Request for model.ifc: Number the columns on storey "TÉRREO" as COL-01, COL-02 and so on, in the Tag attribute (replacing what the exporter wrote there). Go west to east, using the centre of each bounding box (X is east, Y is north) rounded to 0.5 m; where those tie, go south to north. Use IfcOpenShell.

First a look at what the model holds.

```python
import ifcopenshell
import ifcopenshell.util.element
import ifcopenshell.util.placement

model = ifcopenshell.open("model.ifc")
print(model.schema)
storey = next(s for s in model.by_type("IfcBuildingStorey") if s.Name == "TÉRREO")
columns = [e for e in ifcopenshell.util.element.get_decomposition(storey) if e.is_a("IfcColumn")]
for e in sorted(columns, key=lambda e: e.id()):
    origin = ifcopenshell.util.placement.get_local_placement(e.ObjectPlacement)[:3, 3]
    print(e.id(), e.Tag, e.Name, origin.round(2) + 0.0, sep=" | ")
```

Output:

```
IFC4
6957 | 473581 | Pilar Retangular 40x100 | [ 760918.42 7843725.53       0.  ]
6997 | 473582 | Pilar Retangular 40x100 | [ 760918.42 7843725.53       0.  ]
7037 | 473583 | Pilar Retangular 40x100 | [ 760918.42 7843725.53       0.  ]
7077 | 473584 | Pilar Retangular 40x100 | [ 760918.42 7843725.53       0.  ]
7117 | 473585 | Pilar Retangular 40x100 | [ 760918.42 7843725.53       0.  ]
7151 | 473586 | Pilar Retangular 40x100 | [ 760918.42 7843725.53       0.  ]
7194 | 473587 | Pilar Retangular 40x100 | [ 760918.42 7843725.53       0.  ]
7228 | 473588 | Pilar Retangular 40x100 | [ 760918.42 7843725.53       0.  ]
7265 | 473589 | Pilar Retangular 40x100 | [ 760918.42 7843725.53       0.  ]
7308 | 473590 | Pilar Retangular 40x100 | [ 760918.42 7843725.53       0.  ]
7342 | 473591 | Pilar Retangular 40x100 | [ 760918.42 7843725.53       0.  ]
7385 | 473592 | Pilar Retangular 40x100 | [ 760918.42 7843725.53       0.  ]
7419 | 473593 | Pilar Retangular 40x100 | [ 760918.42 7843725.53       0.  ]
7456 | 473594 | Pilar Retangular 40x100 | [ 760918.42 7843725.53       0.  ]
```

```python
import ifcopenshell
import ifcopenshell.geom
import ifcopenshell.util.element
import ifcopenshell.util.shape

model = ifcopenshell.open("model.ifc")
settings = ifcopenshell.geom.settings()
settings.set("use-world-coords", True)


def centre(element):
    shape = ifcopenshell.geom.create_shape(settings, element)
    return ifcopenshell.util.shape.get_bbox_centroid(shape.geometry)


storey = next(s for s in model.by_type("IfcBuildingStorey") if s.Name == "TÉRREO")
columns = [e for e in ifcopenshell.util.element.get_decomposition(storey) if e.is_a("IfcColumn")]

# Insertion points can sit at a corner or the storey origin, so sort by the geometry (in metres).
centres = {e: centre(e) for e in columns}
columns.sort(key=lambda e: (round(centres[e][0] / 0.5), centres[e][1]))

for i, e in enumerate(columns, start=1):
    number = f"COL-{i:02d}"
    e.Tag = number
    print(e.id(), number)

model.write("model_v2.ifc")
```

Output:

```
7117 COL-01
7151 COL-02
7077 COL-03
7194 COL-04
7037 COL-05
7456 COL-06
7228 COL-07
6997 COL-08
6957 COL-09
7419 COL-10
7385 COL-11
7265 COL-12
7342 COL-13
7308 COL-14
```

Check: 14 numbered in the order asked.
